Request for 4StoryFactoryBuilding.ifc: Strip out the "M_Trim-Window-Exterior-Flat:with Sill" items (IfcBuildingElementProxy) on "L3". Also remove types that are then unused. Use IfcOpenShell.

First a look at what the model holds.

```python
import ifcopenshell
import ifcopenshell.util.element

model = ifcopenshell.open("4StoryFactoryBuilding.ifc")
print(model.schema)
storey = next(s for s in model.by_type("IfcBuildingStorey") if s.Name == "L3")
proxies = [e for e in ifcopenshell.util.element.get_decomposition(storey) if e.is_a("IfcBuildingElementProxy")]
seen = {}
for e in proxies:
    element_type = ifcopenshell.util.element.get_type(e)
    name = element_type.Name if element_type not in (None, e) else None
    seen[name] = seen.get(name, 0) + 1
for name, count in sorted(seen.items(), key=str):
    print(count, "x", name)
```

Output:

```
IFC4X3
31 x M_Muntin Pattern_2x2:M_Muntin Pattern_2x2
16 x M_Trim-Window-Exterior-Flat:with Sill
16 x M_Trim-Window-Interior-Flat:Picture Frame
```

```python
import ifcopenshell
import ifcopenshell.api.root
import ifcopenshell.util.element

model = ifcopenshell.open("4StoryFactoryBuilding.ifc")

storey = next(s for s in model.by_type("IfcBuildingStorey") if s.Name == "L3")
proxies = [e for e in ifcopenshell.util.element.get_decomposition(storey) if e.is_a("IfcBuildingElementProxy")]
targets = [e for e in proxies if (t := ifcopenshell.util.element.get_type(e)) not in (None, e) and t.Name == "M_Trim-Window-Exterior-Flat:with Sill"]
types = {ifcopenshell.util.element.get_type(e) for e in targets} - {None, *targets}

for e in targets:
    ifcopenshell.api.root.remove_product(model, product=e)
print(len(targets), "removed")

unused = [t for t in types if not ifcopenshell.util.element.get_types(t)]
for t in unused:
    ifcopenshell.api.root.remove_product(model, product=t)
print(len(unused), "unused types removed")

model.write("4StoryFactoryBuilding_edited.ifc")
```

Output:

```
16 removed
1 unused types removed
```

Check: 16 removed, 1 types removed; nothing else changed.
